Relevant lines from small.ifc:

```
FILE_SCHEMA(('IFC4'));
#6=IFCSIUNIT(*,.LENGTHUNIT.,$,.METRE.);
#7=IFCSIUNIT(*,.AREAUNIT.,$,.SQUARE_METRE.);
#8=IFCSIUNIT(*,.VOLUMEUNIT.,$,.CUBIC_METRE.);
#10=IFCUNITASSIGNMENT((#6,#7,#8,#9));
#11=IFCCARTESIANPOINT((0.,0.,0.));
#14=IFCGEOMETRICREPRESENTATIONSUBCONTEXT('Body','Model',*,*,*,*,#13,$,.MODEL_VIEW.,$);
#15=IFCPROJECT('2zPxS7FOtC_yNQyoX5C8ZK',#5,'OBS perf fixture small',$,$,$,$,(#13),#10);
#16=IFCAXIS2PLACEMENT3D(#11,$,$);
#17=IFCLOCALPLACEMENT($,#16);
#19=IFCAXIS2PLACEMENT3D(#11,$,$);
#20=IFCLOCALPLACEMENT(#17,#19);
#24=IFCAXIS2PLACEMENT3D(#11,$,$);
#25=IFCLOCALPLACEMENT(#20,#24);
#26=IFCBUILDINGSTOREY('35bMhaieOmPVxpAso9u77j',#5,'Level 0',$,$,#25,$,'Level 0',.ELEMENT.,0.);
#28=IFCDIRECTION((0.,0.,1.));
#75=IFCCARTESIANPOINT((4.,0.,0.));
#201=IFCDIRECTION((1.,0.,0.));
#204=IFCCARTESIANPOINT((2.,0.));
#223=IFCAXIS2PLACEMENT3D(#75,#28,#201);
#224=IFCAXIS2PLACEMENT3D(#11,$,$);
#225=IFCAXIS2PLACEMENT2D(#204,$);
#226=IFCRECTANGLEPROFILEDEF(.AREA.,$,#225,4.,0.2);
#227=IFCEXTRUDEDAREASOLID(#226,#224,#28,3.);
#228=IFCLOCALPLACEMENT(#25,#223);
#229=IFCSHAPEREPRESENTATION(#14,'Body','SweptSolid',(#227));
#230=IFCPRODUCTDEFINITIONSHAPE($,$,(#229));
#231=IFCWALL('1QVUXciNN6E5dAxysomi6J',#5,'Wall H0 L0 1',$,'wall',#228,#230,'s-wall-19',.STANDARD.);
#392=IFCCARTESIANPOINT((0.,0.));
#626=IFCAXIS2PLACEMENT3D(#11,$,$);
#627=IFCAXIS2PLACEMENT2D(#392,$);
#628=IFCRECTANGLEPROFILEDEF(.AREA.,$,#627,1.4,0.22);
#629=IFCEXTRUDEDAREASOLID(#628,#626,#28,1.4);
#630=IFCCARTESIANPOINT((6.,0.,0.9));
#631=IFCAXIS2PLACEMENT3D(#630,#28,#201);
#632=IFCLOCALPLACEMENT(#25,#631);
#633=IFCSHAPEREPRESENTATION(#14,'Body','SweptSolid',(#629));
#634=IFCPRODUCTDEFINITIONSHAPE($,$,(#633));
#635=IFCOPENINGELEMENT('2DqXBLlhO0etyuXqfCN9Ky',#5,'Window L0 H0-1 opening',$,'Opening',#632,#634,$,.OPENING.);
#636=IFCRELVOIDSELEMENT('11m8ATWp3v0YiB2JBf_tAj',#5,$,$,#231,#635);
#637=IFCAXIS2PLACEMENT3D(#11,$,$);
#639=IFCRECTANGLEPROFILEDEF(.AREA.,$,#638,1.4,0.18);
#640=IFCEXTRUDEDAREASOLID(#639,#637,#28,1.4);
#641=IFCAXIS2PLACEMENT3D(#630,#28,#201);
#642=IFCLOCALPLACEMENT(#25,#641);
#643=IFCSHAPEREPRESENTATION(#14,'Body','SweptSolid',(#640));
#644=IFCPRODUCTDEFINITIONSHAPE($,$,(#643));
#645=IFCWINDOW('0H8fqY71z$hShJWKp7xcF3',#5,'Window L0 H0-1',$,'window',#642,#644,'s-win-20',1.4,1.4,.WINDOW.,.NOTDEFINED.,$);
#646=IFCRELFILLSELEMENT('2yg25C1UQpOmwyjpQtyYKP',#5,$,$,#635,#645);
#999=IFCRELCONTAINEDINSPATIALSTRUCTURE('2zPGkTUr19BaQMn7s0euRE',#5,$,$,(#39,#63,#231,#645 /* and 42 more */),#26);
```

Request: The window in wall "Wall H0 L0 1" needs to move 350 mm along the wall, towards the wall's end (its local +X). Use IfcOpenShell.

```python
import ifcopenshell
import ifcopenshell.api.geometry
import ifcopenshell.util.placement
import ifcopenshell.util.unit

model = ifcopenshell.open("small.ifc")
unit_scale = ifcopenshell.util.unit.calculate_unit_scale(model)

window = model.by_id(645)
opening = window.FillsVoids[0].RelatingOpeningElement
wall = opening.VoidsElements[0].RelatingBuildingElement

wall_matrix = ifcopenshell.util.placement.get_local_placement(wall.ObjectPlacement)
shift = wall_matrix[:3, 0] * 0.35 / unit_scale
before = ifcopenshell.util.placement.get_local_placement(window.ObjectPlacement)[:3, 3].copy()

# The window is not placed relative to its opening, so move both.
for product in (opening, window):
    matrix = ifcopenshell.util.placement.get_local_placement(product.ObjectPlacement)
    matrix[:3, 3] += shift
    ifcopenshell.api.geometry.edit_object_placement(model, product=product, matrix=matrix, is_si=False)

after = ifcopenshell.util.placement.get_local_placement(window.ObjectPlacement)[:3, 3]
print("window moved by", (after - before).round(3) + 0.0)

model.write("small_v2.ifc")
```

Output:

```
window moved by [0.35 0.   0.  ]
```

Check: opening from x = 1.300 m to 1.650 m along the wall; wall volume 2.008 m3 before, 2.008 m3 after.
